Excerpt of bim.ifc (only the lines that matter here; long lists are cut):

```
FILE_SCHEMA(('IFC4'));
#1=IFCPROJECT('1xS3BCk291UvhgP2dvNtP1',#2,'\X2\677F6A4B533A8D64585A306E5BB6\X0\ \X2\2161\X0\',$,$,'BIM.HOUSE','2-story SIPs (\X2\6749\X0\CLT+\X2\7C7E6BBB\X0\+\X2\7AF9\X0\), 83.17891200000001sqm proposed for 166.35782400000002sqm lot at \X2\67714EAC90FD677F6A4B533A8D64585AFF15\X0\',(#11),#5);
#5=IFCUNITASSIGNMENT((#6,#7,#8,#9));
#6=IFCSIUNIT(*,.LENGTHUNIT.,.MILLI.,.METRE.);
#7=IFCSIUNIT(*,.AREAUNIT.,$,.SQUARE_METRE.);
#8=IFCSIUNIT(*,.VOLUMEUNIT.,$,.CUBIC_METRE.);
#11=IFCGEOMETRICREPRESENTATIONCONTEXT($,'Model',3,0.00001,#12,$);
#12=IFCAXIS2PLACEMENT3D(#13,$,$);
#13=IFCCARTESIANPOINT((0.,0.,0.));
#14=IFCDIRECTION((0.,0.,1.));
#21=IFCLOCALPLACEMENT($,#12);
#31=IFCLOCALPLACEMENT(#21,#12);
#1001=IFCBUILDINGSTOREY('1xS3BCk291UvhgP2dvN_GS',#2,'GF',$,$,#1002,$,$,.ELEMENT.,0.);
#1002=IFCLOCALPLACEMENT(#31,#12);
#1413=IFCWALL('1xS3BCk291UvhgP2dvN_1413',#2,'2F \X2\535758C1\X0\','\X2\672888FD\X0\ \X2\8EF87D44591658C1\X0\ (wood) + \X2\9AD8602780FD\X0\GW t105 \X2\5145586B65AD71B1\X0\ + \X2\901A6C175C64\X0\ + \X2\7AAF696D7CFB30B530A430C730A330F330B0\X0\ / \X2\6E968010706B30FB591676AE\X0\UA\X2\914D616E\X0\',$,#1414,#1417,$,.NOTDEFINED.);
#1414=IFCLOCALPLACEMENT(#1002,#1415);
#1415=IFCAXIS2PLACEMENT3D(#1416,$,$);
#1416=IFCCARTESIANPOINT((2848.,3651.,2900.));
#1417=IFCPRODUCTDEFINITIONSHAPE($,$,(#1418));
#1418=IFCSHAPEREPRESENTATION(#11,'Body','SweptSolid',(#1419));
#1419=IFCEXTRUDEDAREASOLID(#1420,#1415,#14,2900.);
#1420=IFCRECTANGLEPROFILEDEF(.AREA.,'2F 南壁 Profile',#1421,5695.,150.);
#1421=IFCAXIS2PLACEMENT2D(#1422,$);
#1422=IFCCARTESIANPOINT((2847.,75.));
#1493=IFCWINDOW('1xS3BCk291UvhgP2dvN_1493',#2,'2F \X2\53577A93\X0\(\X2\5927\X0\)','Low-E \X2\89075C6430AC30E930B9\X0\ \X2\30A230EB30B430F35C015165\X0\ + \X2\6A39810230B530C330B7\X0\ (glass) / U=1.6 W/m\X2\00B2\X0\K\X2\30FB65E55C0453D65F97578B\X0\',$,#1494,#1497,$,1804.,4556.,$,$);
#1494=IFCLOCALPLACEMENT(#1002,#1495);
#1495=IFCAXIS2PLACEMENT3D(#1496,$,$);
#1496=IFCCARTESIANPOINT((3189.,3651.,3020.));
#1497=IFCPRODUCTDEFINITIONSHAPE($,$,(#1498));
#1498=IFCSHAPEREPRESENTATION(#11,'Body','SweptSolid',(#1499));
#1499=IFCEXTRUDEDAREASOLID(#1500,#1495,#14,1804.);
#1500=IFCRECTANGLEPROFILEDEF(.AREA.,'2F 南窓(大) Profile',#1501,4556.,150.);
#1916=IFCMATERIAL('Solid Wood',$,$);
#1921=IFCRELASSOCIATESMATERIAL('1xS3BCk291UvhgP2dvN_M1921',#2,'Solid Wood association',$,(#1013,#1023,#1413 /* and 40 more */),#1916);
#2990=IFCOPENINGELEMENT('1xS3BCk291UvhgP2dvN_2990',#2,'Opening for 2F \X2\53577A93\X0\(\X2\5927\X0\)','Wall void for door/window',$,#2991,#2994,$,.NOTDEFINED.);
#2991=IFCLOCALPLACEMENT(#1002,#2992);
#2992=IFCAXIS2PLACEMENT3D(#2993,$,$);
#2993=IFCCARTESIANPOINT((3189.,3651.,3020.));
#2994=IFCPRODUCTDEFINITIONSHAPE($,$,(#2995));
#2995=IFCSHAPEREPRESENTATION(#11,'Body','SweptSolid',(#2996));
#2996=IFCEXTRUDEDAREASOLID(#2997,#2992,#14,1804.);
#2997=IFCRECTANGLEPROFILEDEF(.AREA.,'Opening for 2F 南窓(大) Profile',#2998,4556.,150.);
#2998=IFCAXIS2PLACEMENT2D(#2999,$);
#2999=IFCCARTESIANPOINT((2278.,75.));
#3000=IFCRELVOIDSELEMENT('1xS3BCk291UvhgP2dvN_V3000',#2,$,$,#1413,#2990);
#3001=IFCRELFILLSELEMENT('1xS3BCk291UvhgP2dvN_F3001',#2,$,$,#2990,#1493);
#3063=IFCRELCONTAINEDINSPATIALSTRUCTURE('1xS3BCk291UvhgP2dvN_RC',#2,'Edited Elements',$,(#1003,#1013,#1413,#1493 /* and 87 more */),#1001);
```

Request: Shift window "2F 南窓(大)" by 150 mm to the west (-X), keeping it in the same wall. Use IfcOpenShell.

```python
import ifcopenshell
import ifcopenshell.api.geometry
import ifcopenshell.util.placement
import ifcopenshell.util.unit

model = ifcopenshell.open("bim.ifc")
unit_scale = ifcopenshell.util.unit.calculate_unit_scale(model)

window = model.by_guid("1xS3BCk291UvhgP2dvN_1493")
opening = window.FillsVoids[0].RelatingOpeningElement
wall = opening.VoidsElements[0].RelatingBuildingElement

wall_matrix = ifcopenshell.util.placement.get_local_placement(wall.ObjectPlacement)
shift = wall_matrix[:3, 0] * -0.15 / unit_scale
before = ifcopenshell.util.placement.get_local_placement(window.ObjectPlacement)[:3, 3].copy()

# The window is not placed relative to its opening, so move both.
for product in (opening, window):
    matrix = ifcopenshell.util.placement.get_local_placement(product.ObjectPlacement)
    matrix[:3, 3] += shift
    ifcopenshell.api.geometry.edit_object_placement(model, product=product, matrix=matrix, is_si=False)

after = ifcopenshell.util.placement.get_local_placement(window.ObjectPlacement)[:3, 3]
print("window moved by", (after - before).round(3) + 0.0)

model.write("bim-out.ifc")
```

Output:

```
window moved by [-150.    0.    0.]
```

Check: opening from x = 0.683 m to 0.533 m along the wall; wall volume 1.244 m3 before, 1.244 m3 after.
